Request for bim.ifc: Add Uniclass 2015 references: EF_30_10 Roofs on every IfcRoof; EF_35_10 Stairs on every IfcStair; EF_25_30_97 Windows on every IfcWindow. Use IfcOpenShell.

First a look at what the model holds.

```python
import ifcopenshell

model = ifcopenshell.open("bim.ifc")
print(model.schema)
print("classifications:", [c.Name for c in model.by_type("IfcClassification")])
for ifc_class in ("IfcDoor", "IfcRoof", "IfcStair", "IfcWall", "IfcWindow"):
    print(ifc_class, len(model.by_type(ifc_class)))
```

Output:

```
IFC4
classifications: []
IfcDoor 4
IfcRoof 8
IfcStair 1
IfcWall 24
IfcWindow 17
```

```python
import ifcopenshell
import ifcopenshell.api.classification

model = ifcopenshell.open("bim.ifc")

system = ifcopenshell.api.classification.add_classification(model, classification="Uniclass 2015")

codes = {
    "IfcRoof": ("EF_30_10", "Roofs"),
    "IfcStair": ("EF_35_10", "Stairs"),
    "IfcWindow": ("EF_25_30_97", "Windows"),
}
for ifc_class, (code, name) in codes.items():
    products = model.by_type(ifc_class)
    ifcopenshell.api.classification.add_reference(
        model, products=products, classification=system, identification=code, name=name
    )
    print(code, len(products))

model.write("bim-out.ifc")
```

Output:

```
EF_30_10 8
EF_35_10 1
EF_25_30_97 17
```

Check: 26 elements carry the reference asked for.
